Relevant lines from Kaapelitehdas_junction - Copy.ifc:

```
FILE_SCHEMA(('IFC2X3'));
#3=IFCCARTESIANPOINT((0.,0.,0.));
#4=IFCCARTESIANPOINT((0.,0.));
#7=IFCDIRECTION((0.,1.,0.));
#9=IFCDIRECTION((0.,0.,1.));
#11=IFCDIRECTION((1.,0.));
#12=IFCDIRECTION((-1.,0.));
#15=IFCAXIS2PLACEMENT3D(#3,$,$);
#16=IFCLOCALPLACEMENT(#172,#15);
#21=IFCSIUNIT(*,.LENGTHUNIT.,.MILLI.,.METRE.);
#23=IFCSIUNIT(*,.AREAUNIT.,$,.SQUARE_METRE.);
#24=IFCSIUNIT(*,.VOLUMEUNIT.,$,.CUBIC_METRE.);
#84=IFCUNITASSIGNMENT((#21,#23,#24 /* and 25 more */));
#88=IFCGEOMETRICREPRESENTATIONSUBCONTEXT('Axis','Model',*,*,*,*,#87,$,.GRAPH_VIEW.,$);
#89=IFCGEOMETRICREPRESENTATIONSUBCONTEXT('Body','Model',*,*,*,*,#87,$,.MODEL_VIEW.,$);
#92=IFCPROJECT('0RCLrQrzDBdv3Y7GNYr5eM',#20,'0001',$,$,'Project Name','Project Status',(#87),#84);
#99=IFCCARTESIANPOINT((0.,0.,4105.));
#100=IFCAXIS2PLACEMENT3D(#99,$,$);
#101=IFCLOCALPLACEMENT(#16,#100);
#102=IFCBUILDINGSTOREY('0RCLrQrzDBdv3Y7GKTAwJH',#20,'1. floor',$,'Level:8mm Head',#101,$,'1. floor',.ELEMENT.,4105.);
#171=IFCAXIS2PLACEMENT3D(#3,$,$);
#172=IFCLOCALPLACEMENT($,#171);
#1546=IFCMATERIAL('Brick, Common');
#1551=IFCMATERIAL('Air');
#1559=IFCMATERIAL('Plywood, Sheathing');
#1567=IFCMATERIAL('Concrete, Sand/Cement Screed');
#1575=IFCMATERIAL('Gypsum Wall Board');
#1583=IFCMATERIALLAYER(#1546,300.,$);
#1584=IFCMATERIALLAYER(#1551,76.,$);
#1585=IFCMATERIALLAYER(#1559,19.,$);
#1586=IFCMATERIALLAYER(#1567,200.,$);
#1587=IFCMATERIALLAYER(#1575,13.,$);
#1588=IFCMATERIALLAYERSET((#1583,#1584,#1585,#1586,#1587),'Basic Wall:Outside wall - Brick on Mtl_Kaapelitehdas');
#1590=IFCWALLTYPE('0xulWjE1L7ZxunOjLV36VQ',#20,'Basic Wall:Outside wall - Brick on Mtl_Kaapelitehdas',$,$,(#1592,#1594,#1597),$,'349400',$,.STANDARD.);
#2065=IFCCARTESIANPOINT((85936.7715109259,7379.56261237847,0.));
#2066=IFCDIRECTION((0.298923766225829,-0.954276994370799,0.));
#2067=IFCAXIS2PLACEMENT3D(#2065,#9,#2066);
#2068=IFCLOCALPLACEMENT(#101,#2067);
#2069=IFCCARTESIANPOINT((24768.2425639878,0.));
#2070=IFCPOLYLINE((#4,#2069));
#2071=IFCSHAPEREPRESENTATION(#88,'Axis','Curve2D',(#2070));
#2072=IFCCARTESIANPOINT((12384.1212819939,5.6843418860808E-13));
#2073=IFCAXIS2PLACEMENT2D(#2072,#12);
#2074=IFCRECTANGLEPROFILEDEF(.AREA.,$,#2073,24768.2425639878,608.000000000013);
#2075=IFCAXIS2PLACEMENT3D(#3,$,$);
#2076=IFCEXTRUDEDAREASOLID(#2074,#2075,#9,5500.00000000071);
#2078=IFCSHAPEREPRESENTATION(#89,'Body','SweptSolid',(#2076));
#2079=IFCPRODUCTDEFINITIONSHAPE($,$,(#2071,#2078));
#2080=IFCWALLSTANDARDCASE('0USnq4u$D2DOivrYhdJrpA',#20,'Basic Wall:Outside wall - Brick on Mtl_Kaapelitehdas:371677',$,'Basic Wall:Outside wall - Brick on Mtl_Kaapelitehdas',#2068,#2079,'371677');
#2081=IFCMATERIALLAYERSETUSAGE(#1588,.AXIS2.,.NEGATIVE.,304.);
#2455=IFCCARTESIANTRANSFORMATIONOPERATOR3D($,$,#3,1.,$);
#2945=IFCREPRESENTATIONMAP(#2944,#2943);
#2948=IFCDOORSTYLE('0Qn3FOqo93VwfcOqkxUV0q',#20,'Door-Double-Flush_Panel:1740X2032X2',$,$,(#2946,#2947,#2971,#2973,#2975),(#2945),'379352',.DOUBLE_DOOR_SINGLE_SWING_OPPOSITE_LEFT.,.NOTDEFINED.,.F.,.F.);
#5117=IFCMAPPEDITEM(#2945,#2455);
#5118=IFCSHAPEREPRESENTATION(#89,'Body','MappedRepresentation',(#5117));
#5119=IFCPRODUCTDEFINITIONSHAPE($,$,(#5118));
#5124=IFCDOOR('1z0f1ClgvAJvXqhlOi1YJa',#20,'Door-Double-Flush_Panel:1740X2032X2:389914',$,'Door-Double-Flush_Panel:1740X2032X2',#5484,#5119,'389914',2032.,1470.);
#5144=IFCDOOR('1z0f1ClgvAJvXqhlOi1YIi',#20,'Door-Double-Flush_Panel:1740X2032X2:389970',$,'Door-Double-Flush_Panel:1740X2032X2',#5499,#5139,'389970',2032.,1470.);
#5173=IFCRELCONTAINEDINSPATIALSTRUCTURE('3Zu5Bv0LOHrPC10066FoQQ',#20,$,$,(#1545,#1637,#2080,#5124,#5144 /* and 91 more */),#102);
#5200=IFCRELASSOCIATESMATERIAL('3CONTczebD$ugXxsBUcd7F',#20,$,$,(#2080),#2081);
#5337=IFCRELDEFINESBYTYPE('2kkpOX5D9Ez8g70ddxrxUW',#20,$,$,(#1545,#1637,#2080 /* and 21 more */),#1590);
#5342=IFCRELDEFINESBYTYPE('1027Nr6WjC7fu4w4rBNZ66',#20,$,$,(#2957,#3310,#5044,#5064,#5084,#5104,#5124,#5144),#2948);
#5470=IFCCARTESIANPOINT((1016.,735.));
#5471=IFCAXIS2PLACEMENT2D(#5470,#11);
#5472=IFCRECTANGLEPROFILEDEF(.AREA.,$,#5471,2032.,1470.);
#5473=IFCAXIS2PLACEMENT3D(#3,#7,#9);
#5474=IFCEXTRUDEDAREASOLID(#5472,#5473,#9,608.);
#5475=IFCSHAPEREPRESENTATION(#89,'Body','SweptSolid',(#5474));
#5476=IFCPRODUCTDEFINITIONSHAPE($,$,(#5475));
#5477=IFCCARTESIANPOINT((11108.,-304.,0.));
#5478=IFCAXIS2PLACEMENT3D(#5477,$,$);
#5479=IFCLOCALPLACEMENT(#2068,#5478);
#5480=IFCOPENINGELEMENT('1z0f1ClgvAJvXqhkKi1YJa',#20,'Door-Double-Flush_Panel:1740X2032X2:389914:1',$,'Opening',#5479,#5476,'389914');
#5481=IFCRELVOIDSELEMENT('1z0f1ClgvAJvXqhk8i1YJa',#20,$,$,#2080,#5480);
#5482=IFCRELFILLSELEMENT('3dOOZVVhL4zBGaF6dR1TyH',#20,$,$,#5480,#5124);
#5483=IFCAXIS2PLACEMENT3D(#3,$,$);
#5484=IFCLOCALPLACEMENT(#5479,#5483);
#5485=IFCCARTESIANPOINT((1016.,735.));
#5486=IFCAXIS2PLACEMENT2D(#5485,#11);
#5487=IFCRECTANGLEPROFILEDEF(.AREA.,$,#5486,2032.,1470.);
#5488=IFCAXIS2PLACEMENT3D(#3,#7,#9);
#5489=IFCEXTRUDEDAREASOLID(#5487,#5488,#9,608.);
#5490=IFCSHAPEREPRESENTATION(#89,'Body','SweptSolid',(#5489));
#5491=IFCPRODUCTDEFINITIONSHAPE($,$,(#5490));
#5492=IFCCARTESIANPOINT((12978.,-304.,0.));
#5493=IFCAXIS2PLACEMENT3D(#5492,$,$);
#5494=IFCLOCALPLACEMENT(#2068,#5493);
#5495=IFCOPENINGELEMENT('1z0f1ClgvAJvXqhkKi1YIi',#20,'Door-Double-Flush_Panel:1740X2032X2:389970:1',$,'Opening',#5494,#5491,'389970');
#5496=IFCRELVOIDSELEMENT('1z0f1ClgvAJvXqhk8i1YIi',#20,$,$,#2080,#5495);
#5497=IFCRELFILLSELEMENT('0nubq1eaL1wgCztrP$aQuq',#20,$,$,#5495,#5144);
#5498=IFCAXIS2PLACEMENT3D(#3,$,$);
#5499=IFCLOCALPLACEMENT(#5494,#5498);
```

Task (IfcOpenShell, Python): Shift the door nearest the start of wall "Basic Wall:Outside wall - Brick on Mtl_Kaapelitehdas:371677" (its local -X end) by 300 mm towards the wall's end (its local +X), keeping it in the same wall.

```python
import ifcopenshell
import ifcopenshell.api.geometry
import ifcopenshell.util.placement
import ifcopenshell.util.unit

model = ifcopenshell.open("Kaapelitehdas_junction - Copy.ifc")
unit_scale = ifcopenshell.util.unit.calculate_unit_scale(model)

door = model.by_guid("1z0f1ClgvAJvXqhlOi1YJa")
opening = door.FillsVoids[0].RelatingOpeningElement
wall = opening.VoidsElements[0].RelatingBuildingElement

wall_matrix = ifcopenshell.util.placement.get_local_placement(wall.ObjectPlacement)
shift = wall_matrix[:3, 0] * 0.3 / unit_scale
before = ifcopenshell.util.placement.get_local_placement(door.ObjectPlacement)[:3, 3].copy()

# The door is placed relative to its opening, so it follows when the opening moves.
matrix = ifcopenshell.util.placement.get_local_placement(opening.ObjectPlacement)
matrix[:3, 3] += shift
ifcopenshell.api.geometry.edit_object_placement(
    model, product=opening, matrix=matrix, is_si=False, should_transform_children=True
)

after = ifcopenshell.util.placement.get_local_placement(door.ObjectPlacement)[:3, 3]
print("door moved by", (after - before).round(3) + 0.0)

model.write("Kaapelitehdas_junction - Copy_edited.ifc")
```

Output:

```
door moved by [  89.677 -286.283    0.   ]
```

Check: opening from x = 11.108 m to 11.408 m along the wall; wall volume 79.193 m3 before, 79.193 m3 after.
